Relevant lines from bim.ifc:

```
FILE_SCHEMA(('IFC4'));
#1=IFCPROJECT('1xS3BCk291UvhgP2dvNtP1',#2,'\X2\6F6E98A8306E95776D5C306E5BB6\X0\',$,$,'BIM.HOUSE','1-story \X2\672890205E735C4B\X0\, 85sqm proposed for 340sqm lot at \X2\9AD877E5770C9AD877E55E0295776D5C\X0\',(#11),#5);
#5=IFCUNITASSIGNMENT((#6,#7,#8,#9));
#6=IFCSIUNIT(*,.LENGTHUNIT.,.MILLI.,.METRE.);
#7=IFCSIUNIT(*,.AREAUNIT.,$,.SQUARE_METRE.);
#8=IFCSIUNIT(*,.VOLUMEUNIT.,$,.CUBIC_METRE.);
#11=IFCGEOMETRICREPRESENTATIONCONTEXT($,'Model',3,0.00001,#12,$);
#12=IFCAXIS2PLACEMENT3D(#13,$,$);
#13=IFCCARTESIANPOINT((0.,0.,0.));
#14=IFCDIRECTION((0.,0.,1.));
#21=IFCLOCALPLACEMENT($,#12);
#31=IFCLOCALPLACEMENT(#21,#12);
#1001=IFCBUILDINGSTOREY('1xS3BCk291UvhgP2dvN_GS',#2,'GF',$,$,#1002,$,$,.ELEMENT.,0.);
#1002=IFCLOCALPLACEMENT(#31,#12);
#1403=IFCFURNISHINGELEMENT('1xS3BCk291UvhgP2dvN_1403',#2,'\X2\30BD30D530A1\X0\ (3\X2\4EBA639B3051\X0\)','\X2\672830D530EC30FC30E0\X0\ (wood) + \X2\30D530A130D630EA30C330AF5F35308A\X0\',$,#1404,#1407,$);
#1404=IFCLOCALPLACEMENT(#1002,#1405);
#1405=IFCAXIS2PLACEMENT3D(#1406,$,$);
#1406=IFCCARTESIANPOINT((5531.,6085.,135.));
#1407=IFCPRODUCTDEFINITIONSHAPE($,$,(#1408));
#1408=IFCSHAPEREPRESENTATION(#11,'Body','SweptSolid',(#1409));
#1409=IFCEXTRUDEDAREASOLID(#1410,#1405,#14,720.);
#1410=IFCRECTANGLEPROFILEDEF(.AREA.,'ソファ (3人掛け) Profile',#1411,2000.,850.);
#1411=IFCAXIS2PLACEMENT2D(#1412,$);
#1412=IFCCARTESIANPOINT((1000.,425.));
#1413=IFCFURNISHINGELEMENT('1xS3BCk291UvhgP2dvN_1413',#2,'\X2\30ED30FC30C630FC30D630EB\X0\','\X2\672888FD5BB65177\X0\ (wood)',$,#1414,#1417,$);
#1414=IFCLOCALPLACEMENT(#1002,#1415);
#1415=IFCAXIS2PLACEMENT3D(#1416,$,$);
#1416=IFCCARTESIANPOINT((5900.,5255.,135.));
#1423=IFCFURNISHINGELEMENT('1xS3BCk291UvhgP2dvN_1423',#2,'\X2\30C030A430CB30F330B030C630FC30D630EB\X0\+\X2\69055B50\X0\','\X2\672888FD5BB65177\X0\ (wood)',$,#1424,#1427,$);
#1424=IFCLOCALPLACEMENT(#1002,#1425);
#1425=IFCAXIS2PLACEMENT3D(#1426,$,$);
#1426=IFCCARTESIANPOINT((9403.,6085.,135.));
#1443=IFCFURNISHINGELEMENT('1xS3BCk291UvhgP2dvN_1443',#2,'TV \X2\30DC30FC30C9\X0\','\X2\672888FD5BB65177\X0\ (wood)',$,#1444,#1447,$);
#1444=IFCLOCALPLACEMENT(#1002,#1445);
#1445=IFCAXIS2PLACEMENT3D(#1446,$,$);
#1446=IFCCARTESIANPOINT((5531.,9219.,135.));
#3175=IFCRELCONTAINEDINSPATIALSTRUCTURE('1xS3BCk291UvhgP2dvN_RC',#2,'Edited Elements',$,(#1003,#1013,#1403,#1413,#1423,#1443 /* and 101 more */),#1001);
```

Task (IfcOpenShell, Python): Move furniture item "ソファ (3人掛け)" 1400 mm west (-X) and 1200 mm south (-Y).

```python
import ifcopenshell
import ifcopenshell.api.geometry
import ifcopenshell.util.placement

model = ifcopenshell.open("bim.ifc")

item = model.by_guid("1xS3BCk291UvhgP2dvN_1403")
matrix = ifcopenshell.util.placement.get_local_placement(item.ObjectPlacement)
matrix[0, 3] -= 1400.0
matrix[1, 3] -= 1200.0
ifcopenshell.api.geometry.edit_object_placement(model, product=item, matrix=matrix, is_si=False)

print(ifcopenshell.util.placement.get_local_placement(item.ObjectPlacement).round(3) + 0.0)

model.write("bim_rev.ifc")
```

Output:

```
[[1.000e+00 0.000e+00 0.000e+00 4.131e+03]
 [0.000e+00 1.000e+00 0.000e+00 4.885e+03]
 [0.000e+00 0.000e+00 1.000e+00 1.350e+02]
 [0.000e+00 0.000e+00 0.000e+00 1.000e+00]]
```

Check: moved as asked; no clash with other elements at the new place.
